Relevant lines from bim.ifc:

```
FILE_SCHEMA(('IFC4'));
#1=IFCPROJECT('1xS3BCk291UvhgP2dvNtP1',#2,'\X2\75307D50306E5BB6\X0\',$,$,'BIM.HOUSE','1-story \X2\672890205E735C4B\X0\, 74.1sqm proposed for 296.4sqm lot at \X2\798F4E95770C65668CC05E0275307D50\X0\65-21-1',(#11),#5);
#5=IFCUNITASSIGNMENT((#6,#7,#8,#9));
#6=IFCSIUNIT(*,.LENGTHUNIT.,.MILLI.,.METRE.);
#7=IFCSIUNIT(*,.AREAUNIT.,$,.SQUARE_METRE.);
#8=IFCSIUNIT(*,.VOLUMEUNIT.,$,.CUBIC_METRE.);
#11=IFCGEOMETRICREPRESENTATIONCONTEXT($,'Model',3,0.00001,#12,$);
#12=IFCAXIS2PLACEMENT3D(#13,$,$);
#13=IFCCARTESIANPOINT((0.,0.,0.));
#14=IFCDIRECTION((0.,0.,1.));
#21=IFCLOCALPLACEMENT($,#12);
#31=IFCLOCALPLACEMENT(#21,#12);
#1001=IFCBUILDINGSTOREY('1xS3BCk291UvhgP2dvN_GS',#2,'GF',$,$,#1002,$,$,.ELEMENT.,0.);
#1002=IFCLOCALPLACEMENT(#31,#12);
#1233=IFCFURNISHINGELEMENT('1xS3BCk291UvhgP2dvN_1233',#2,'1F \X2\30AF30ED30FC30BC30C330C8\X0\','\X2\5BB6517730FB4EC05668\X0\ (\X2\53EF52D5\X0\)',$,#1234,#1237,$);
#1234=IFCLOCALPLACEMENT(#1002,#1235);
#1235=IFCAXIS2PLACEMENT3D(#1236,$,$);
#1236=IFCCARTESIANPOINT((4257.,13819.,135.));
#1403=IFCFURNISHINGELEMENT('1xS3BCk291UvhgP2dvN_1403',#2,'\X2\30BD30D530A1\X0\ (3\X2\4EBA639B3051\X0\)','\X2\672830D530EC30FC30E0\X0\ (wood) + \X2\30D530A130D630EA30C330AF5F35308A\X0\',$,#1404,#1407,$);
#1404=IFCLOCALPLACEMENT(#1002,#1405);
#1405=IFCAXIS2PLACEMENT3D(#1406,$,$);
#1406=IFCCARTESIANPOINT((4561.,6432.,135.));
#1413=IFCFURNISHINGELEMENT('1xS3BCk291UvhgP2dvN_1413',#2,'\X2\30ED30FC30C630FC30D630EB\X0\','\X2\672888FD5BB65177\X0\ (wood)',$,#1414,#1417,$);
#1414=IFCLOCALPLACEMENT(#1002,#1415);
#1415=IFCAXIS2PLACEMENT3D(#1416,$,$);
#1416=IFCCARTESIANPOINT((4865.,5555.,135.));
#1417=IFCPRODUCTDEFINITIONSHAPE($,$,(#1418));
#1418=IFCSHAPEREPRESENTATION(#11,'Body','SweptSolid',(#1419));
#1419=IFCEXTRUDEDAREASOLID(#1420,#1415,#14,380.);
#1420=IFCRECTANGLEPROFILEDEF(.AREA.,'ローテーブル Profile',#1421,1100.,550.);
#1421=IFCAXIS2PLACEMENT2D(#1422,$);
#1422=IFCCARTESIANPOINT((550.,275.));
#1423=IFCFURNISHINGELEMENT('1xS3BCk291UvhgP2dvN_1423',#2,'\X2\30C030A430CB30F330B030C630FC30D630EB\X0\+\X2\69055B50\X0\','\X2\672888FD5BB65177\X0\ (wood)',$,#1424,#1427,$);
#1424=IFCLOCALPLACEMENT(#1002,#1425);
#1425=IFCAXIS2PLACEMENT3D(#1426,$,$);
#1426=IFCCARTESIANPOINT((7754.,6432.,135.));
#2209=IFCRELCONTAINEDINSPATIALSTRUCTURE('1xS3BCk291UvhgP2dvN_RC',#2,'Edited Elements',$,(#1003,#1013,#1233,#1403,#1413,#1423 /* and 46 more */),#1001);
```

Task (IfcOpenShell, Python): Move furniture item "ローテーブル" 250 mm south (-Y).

```python
import ifcopenshell
import ifcopenshell.api.geometry
import ifcopenshell.util.placement
import ifcopenshell.util.unit

model = ifcopenshell.open("bim.ifc")
unit_scale = ifcopenshell.util.unit.calculate_unit_scale(model)

item = model.by_guid("1xS3BCk291UvhgP2dvN_1413")
matrix = ifcopenshell.util.placement.get_local_placement(item.ObjectPlacement)
matrix[1, 3] -= 0.25 / unit_scale
ifcopenshell.api.geometry.edit_object_placement(model, product=item, matrix=matrix, is_si=False)

print(ifcopenshell.util.placement.get_local_placement(item.ObjectPlacement).round(3) + 0.0)

model.write("bim_rev.ifc")
```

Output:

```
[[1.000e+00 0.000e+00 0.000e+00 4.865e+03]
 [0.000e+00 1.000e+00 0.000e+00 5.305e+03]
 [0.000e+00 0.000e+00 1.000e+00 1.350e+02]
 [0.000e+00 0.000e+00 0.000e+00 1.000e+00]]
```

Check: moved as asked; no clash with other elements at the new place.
